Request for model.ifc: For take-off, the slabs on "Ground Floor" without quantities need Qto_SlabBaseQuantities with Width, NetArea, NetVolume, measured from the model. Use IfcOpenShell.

First a look at what the model holds.

```python
import ifcopenshell
import ifcopenshell.util.element
import ifcopenshell.util.unit

model = ifcopenshell.open("model.ifc")
print(model.schema)
for unit_type in ("LENGTHUNIT", "AREAUNIT", "VOLUMEUNIT"):
    print(unit_type, ifcopenshell.util.unit.calculate_unit_scale(model, unit_type))
storey = next(s for s in model.by_type("IfcBuildingStorey") if s.Name == "Ground Floor")
slabs = [e for e in ifcopenshell.util.element.get_decomposition(storey) if e.is_a("IfcSlab")]
for e in sorted(slabs, key=lambda e: e.id()):
    print(e.id(), e.is_a(), e.Name, list(ifcopenshell.util.element.get_psets(e, qtos_only=True)), sep=" | ")
```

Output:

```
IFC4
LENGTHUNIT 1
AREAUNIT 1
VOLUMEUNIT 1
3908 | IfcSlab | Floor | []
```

```python
import ifcopenshell
import ifcopenshell.api.pset
import ifcopenshell.geom
import ifcopenshell.util.element
import ifcopenshell.util.shape
import ifcopenshell.util.unit

model = ifcopenshell.open("model.ifc")
unit_scale = ifcopenshell.util.unit.calculate_unit_scale(model)
area_scale = ifcopenshell.util.unit.calculate_unit_scale(model, "AREAUNIT")
volume_scale = ifcopenshell.util.unit.calculate_unit_scale(model, "VOLUMEUNIT")
settings = ifcopenshell.geom.settings()

storey = next(s for s in model.by_type("IfcBuildingStorey") if s.Name == "Ground Floor")
slabs = [e for e in ifcopenshell.util.element.get_decomposition(storey) if e.is_a("IfcSlab")]

for e in sorted(slabs, key=lambda e: e.id()):
    if ifcopenshell.util.element.get_psets(e, qtos_only=True, should_inherit=False):
        continue
    # Geometry comes back in metres, in the element's own axes.
    shape = ifcopenshell.geom.create_shape(settings, e)
    values = {
        "Width": ifcopenshell.util.shape.get_z(shape.geometry) / unit_scale,
        "NetArea": ifcopenshell.util.shape.get_footprint_area(shape.geometry) / area_scale,
        "NetVolume": ifcopenshell.util.shape.get_volume(shape.geometry) / volume_scale,
    }
    qto = ifcopenshell.api.pset.add_qto(model, product=e, name="Qto_SlabBaseQuantities")
    ifcopenshell.api.pset.edit_qto(model, qto=qto, properties=values)
    print(e.id(), {k: round(v, 3) for k, v in values.items()})

model.write("model_updated.ifc")
```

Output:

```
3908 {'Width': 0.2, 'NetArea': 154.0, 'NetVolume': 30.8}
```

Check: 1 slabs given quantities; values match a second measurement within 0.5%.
